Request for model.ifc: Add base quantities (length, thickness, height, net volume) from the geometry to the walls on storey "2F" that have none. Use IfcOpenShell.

First a look at what the model holds.

```python
import ifcopenshell
import ifcopenshell.util.element
import ifcopenshell.util.unit

model = ifcopenshell.open("model.ifc")
print(model.schema)
for unit_type in ("LENGTHUNIT", "AREAUNIT", "VOLUMEUNIT"):
    print(unit_type, ifcopenshell.util.unit.calculate_unit_scale(model, unit_type))
storey = next(s for s in model.by_type("IfcBuildingStorey") if s.Name == "2F")
walls = [e for e in ifcopenshell.util.element.get_decomposition(storey) if e.is_a("IfcWall")]
for e in sorted(walls, key=lambda e: e.id()):
    print(e.id(), e.is_a(), e.Name, list(ifcopenshell.util.element.get_psets(e, qtos_only=True)), sep=" | ")
```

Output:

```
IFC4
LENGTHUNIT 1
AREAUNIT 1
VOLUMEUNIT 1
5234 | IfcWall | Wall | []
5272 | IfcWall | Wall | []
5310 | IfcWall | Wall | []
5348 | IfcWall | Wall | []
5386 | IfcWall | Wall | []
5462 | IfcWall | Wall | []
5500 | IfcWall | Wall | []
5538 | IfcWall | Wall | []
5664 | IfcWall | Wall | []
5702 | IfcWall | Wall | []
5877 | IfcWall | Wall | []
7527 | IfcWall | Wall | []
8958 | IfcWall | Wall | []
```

```python
import ifcopenshell
import ifcopenshell.api.pset
import ifcopenshell.geom
import ifcopenshell.util.element
import ifcopenshell.util.shape
import ifcopenshell.util.unit

model = ifcopenshell.open("model.ifc")
unit_scale = ifcopenshell.util.unit.calculate_unit_scale(model)
volume_scale = ifcopenshell.util.unit.calculate_unit_scale(model, "VOLUMEUNIT")
settings = ifcopenshell.geom.settings()

storey = next(s for s in model.by_type("IfcBuildingStorey") if s.Name == "2F")
walls = [e for e in ifcopenshell.util.element.get_decomposition(storey) if e.is_a("IfcWall")]

for e in sorted(walls, key=lambda e: e.id()):
    if ifcopenshell.util.element.get_psets(e, qtos_only=True, should_inherit=False):
        continue
    # Geometry comes back in metres, in the element's own axes.
    shape = ifcopenshell.geom.create_shape(settings, e)
    values = {
        "Length": ifcopenshell.util.shape.get_x(shape.geometry) / unit_scale,
        "Width": ifcopenshell.util.shape.get_y(shape.geometry) / unit_scale,
        "Height": ifcopenshell.util.shape.get_z(shape.geometry) / unit_scale,
        "NetVolume": ifcopenshell.util.shape.get_volume(shape.geometry) / volume_scale,
    }
    qto = ifcopenshell.api.pset.add_qto(model, product=e, name="Qto_WallBaseQuantities")
    ifcopenshell.api.pset.edit_qto(model, qto=qto, properties=values)
    print(e.id(), {k: round(v, 3) for k, v in values.items()})

model.write("model_updated.ifc")
```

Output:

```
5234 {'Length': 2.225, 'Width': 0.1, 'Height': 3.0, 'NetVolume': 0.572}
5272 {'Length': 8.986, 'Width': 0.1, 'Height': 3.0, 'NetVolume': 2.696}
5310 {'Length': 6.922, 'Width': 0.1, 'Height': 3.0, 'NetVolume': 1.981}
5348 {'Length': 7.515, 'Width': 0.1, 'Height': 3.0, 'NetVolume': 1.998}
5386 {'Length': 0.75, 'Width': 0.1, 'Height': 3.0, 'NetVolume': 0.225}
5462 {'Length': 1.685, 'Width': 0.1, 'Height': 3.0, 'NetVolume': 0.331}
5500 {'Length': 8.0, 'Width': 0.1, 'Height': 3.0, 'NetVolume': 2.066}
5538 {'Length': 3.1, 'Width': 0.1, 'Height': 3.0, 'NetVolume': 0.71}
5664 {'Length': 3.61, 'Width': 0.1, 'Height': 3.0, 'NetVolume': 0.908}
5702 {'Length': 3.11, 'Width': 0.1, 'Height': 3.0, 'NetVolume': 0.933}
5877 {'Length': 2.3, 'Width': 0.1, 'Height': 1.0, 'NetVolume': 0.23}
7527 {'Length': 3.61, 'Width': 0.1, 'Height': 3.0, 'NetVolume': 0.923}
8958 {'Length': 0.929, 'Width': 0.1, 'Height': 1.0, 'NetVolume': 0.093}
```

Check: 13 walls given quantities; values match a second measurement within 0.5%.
